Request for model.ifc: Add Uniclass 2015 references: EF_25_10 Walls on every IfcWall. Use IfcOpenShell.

First a look at what the model holds.

```python
import ifcopenshell

model = ifcopenshell.open("model.ifc")
print(model.schema)
print("classifications:", [c.Name for c in model.by_type("IfcClassification")])
for ifc_class in ("IfcDoor", "IfcRoof", "IfcStair", "IfcWall", "IfcWindow"):
    print(ifc_class, len(model.by_type(ifc_class)))
```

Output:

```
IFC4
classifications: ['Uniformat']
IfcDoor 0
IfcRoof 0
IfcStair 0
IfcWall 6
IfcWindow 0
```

```python
import ifcopenshell
import ifcopenshell.api.classification

model = ifcopenshell.open("model.ifc")

system = ifcopenshell.api.classification.add_classification(model, classification="Uniclass 2015")

codes = {
    "IfcWall": ("EF_25_10", "Walls"),
}
for ifc_class, (code, name) in codes.items():
    products = model.by_type(ifc_class)
    ifcopenshell.api.classification.add_reference(
        model, products=products, classification=system, identification=code, name=name
    )
    print(code, len(products))

model.write("model-out.ifc")
```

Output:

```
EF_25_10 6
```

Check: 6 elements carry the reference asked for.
